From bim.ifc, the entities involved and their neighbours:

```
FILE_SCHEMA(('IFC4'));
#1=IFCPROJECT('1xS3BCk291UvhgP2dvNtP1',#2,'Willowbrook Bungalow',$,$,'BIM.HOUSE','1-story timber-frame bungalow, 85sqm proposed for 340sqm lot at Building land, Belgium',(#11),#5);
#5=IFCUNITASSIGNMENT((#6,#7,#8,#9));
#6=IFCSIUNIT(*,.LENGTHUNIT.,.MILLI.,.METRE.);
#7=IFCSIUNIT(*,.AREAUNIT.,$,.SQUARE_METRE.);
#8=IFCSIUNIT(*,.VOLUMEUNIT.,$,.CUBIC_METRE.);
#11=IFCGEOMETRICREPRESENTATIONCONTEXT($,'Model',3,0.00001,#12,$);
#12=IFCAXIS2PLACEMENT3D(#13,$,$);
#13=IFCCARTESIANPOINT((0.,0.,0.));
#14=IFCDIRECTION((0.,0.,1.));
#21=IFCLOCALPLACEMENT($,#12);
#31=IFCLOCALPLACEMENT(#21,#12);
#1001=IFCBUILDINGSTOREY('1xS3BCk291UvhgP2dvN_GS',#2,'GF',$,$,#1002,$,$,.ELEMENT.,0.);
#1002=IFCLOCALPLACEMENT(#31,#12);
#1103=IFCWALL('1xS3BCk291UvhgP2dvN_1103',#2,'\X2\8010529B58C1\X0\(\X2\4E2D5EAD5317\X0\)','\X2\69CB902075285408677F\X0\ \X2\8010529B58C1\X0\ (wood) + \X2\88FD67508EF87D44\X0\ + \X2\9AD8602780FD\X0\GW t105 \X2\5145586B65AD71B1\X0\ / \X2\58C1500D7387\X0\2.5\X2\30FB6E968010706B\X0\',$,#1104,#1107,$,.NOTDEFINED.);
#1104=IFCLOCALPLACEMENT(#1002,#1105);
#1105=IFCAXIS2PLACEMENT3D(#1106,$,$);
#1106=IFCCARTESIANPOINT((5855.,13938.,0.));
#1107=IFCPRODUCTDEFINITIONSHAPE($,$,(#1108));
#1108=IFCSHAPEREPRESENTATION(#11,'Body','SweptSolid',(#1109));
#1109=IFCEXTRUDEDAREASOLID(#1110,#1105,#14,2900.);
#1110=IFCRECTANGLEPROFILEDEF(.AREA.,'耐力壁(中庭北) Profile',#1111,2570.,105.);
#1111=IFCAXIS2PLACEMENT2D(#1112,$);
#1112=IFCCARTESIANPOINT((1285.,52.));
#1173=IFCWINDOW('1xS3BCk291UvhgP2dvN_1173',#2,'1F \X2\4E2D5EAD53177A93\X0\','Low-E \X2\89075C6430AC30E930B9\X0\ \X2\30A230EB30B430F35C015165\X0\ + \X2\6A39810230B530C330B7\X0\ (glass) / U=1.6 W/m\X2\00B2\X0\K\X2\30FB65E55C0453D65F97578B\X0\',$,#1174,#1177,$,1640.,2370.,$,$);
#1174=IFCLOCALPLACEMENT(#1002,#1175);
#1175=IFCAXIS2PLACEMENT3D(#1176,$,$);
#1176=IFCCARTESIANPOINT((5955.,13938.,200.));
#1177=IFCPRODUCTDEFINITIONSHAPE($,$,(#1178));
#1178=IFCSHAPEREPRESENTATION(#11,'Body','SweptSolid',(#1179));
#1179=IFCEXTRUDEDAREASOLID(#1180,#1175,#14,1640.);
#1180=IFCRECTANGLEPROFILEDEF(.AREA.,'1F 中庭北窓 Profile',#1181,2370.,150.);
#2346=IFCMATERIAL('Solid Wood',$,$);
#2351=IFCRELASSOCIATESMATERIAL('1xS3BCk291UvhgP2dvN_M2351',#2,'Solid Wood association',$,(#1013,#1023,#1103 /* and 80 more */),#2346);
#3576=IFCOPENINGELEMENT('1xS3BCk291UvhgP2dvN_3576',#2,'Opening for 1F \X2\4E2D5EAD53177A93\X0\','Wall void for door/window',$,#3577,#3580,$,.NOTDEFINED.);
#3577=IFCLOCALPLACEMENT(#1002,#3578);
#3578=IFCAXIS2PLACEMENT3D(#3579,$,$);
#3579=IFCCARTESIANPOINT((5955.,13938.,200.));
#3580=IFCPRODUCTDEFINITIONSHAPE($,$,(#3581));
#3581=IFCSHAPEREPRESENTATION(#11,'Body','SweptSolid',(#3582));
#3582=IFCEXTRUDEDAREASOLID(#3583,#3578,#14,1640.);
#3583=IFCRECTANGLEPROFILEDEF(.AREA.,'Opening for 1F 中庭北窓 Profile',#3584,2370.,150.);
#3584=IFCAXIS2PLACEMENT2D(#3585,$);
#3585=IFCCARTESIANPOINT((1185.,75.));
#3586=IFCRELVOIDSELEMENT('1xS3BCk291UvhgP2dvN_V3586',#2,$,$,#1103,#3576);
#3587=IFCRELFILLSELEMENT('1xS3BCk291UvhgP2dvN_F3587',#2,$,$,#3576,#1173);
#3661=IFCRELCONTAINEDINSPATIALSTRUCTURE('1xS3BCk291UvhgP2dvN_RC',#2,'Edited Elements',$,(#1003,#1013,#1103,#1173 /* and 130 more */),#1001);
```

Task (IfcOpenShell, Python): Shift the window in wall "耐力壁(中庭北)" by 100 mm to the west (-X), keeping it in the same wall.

```python
import ifcopenshell
import ifcopenshell.api.geometry
import ifcopenshell.util.placement

model = ifcopenshell.open("bim.ifc")

window = model.by_guid("1xS3BCk291UvhgP2dvN_1173")
opening = window.FillsVoids[0].RelatingOpeningElement
wall = opening.VoidsElements[0].RelatingBuildingElement

wall_matrix = ifcopenshell.util.placement.get_local_placement(wall.ObjectPlacement)
shift = wall_matrix[:3, 0] * -100.0
before = ifcopenshell.util.placement.get_local_placement(window.ObjectPlacement)[:3, 3].copy()

# The window is not placed relative to its opening, so move both.
for product in (opening, window):
    matrix = ifcopenshell.util.placement.get_local_placement(product.ObjectPlacement)
    matrix[:3, 3] += shift
    ifcopenshell.api.geometry.edit_object_placement(model, product=product, matrix=matrix, is_si=False)

after = ifcopenshell.util.placement.get_local_placement(window.ObjectPlacement)[:3, 3]
print("window moved by", (after - before).round(3) + 0.0)

model.write("bim_rev.ifc")
```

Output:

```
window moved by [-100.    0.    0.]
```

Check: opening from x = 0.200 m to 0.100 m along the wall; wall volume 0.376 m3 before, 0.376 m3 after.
